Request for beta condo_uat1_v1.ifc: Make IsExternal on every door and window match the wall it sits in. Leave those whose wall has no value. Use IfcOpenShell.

First a look at what the model holds.

```python
import ifcopenshell
import ifcopenshell.util.element

model = ifcopenshell.open("beta condo_uat1_v1.ifc")
print(model.schema)
seen = {}
for e in model.by_type("IfcDoor") + model.by_type("IfcWindow"):
    if not e.FillsVoids:
        continue
    host = e.FillsVoids[0].RelatingOpeningElement.VoidsElements[0].RelatingBuildingElement
    own = ifcopenshell.util.element.get_pset(e, f"Pset_{e.is_a()[3:].removesuffix('StandardCase')}Common", "IsExternal")
    wall = ifcopenshell.util.element.get_pset(host, "Pset_WallCommon", "IsExternal")
    seen[e.is_a(), own, wall] = seen.get((e.is_a(), own, wall), 0) + 1
for (cls, own, wall), count in sorted(seen.items(), key=str):
    print(count, cls, "IsExternal:", own, "| host wall:", wall)
```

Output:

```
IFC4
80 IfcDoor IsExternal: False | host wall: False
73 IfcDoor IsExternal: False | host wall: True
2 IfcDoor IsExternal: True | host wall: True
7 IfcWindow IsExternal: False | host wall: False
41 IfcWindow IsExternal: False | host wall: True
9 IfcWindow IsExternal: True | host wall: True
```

```python
import ifcopenshell
import ifcopenshell.api.pset
import ifcopenshell.util.element

model = ifcopenshell.open("beta condo_uat1_v1.ifc")

count = 0
for ifc_class, pset_name in (("IfcDoor", "Pset_DoorCommon"), ("IfcWindow", "Pset_WindowCommon")):
    for e in model.by_type(ifc_class):
        if not e.FillsVoids:
            continue
        host = e.FillsVoids[0].RelatingOpeningElement.VoidsElements[0].RelatingBuildingElement
        external = ifcopenshell.util.element.get_pset(host, "Pset_WallCommon", "IsExternal")
        if external is None or ifcopenshell.util.element.get_pset(e, pset_name, "IsExternal") == external:
            continue
        pset = ifcopenshell.api.pset.add_pset(model, product=e, name=pset_name)
        ifcopenshell.api.pset.edit_pset(model, pset=pset, properties={"IsExternal": external})
        count += 1

print(count, "updated")

model.write("beta condo_uat1_v1_rev.ifc")
```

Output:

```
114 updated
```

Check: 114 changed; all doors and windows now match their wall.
